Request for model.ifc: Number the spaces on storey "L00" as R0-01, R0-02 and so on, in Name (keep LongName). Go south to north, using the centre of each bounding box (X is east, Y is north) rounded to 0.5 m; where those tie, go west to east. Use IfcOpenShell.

First a look at what the model holds.

```python
import ifcopenshell
import ifcopenshell.util.element
import ifcopenshell.util.placement

model = ifcopenshell.open("model.ifc")
print(model.schema)
storey = next(s for s in model.by_type("IfcBuildingStorey") if s.Name == "L00")
spaces = [e for e in ifcopenshell.util.element.get_decomposition(storey) if e.is_a("IfcSpace")]
for e in sorted(spaces, key=lambda e: e.id()):
    origin = ifcopenshell.util.placement.get_local_placement(e.ObjectPlacement)[:3, 3]
    print(e.id(), e.Name, e.LongName, origin.round(2) + 0.0, sep=" | ")
```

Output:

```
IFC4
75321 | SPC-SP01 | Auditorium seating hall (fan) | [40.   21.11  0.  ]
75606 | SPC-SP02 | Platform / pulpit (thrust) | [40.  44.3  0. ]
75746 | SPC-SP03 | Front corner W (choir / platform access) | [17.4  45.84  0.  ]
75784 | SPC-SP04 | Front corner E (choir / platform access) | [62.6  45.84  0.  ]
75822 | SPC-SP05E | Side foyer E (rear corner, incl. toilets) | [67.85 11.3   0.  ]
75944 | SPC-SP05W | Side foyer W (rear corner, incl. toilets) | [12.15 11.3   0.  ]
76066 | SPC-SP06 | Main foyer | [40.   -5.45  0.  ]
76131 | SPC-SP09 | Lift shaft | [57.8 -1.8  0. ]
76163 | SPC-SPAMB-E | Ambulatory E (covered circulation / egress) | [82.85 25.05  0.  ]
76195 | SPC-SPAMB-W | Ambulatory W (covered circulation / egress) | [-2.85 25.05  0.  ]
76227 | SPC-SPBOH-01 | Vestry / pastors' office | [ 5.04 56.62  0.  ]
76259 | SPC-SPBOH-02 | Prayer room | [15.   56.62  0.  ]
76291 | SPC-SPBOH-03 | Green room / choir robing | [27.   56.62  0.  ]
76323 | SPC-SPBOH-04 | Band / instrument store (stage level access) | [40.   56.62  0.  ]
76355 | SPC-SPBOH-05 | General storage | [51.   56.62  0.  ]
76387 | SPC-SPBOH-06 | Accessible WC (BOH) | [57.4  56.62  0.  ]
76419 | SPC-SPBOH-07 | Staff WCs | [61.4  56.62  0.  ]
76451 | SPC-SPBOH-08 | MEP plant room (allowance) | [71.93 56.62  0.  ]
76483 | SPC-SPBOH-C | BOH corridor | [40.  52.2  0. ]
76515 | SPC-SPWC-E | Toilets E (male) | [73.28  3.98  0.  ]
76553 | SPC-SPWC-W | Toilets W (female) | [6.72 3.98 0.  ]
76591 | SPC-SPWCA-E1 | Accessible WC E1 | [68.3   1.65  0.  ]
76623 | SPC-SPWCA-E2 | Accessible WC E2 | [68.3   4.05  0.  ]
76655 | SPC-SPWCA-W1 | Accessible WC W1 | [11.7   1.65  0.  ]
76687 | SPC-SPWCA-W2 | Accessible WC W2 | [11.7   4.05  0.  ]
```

```python
import ifcopenshell
import ifcopenshell.geom
import ifcopenshell.util.element
import ifcopenshell.util.shape

model = ifcopenshell.open("model.ifc")
settings = ifcopenshell.geom.settings()
settings.set("use-world-coords", True)


def centre(element):
    shape = ifcopenshell.geom.create_shape(settings, element)
    return ifcopenshell.util.shape.get_bbox_centroid(shape.geometry)


storey = next(s for s in model.by_type("IfcBuildingStorey") if s.Name == "L00")
spaces = [e for e in ifcopenshell.util.element.get_decomposition(storey) if e.is_a("IfcSpace")]

# Insertion points can sit at a corner or the storey origin, so sort by the geometry (in metres).
centres = {e: centre(e) for e in spaces}
spaces.sort(key=lambda e: (round(centres[e][1] / 0.5), centres[e][0]))

for i, e in enumerate(spaces, start=1):
    number = f"R0-{i:02d}"
    e.Name = number
    print(e.id(), number)

model.write("model_edited.ifc")
```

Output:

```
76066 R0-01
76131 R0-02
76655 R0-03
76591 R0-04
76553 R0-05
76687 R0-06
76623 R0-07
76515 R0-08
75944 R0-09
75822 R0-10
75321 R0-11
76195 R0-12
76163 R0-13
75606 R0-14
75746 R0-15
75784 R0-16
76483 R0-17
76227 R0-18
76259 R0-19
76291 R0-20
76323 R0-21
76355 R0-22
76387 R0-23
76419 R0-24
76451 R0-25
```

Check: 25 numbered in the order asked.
